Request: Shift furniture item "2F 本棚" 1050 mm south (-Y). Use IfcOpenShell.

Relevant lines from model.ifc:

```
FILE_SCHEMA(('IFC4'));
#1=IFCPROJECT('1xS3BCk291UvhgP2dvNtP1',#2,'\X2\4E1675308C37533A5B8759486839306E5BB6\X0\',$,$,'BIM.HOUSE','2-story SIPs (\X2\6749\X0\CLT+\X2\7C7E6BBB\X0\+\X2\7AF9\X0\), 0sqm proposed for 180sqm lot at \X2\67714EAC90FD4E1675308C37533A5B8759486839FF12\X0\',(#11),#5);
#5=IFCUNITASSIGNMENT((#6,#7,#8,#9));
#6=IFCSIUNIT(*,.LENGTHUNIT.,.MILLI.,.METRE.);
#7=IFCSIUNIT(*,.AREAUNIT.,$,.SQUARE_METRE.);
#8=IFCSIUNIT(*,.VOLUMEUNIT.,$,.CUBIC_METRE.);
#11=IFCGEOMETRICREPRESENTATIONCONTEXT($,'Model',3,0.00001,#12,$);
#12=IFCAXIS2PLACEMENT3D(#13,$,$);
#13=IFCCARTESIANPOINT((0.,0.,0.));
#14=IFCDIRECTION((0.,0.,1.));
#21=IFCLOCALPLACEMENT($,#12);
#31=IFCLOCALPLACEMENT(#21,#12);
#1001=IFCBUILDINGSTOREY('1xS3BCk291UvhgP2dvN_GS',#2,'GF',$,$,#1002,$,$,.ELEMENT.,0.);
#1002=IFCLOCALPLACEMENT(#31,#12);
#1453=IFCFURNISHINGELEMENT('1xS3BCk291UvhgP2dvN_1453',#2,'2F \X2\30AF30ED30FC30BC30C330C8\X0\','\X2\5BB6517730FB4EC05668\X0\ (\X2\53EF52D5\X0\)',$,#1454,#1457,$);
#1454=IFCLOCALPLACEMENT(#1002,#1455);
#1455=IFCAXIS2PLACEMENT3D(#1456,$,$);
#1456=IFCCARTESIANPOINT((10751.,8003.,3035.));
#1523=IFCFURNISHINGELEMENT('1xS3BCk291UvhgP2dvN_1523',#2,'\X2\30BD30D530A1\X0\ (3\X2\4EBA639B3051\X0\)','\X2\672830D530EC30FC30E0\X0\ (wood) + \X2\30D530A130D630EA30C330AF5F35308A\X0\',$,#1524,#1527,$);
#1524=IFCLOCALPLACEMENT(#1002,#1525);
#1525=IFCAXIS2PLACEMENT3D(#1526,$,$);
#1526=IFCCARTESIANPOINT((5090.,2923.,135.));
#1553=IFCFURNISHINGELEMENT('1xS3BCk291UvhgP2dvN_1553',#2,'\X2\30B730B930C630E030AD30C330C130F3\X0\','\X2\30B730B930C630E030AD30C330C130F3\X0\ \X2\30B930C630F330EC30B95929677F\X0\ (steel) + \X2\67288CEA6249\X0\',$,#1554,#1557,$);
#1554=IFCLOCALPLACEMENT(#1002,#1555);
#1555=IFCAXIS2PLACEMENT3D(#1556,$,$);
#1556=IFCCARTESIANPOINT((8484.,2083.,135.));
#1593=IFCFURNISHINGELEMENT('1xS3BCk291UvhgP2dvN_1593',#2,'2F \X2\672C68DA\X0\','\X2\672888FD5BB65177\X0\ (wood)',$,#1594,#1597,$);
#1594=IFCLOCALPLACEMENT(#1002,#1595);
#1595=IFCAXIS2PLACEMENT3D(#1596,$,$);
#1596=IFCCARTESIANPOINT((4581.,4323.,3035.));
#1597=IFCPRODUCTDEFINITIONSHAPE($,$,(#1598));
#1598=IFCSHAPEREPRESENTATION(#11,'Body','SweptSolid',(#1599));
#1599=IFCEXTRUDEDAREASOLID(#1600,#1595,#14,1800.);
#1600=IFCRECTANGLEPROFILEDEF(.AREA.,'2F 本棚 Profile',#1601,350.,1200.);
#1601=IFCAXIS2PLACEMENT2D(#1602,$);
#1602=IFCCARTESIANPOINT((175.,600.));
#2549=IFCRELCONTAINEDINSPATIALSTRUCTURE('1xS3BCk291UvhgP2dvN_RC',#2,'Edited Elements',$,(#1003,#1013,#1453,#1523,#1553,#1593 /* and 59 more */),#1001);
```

```python
import ifcopenshell
import ifcopenshell.api.geometry
import ifcopenshell.util.placement
import ifcopenshell.util.unit

model = ifcopenshell.open("model.ifc")
unit_scale = ifcopenshell.util.unit.calculate_unit_scale(model)

item = model.by_id(1593)
matrix = ifcopenshell.util.placement.get_local_placement(item.ObjectPlacement)
matrix[1, 3] -= 1.05 / unit_scale
ifcopenshell.api.geometry.edit_object_placement(model, product=item, matrix=matrix, is_si=False)

print(ifcopenshell.util.placement.get_local_placement(item.ObjectPlacement).round(3) + 0.0)

model.write("model-out.ifc")
```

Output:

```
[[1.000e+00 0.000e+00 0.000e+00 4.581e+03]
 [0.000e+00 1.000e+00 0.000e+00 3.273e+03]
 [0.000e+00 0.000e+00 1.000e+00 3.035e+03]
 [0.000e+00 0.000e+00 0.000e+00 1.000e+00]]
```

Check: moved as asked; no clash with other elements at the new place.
